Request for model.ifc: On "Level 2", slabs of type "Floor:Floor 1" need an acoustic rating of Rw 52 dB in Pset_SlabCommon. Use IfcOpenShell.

First a look at what the model holds.

```python
import ifcopenshell
import ifcopenshell.util.element

model = ifcopenshell.open("model.ifc")
print(model.schema)
storey = next(s for s in model.by_type("IfcBuildingStorey") if s.Name == "Level 2")
slabs = [e for e in ifcopenshell.util.element.get_decomposition(storey) if e.is_a("IfcSlab")]
seen = {}
for e in slabs:
    element_type = ifcopenshell.util.element.get_type(e)
    key = (element_type.Name if element_type != e and element_type else None, ifcopenshell.util.element.get_pset(e, "Pset_SlabCommon", "AcousticRating"))
    seen[key] = seen.get(key, 0) + 1
for (name, value), count in sorted(seen.items(), key=str):
    print(count, "x", name, "|", value)
```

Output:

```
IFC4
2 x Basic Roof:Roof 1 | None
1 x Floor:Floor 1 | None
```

```python
import ifcopenshell
import ifcopenshell.api.pset
import ifcopenshell.util.element

model = ifcopenshell.open("model.ifc")

storey = next(s for s in model.by_type("IfcBuildingStorey") if s.Name == "Level 2")
slabs = [e for e in ifcopenshell.util.element.get_decomposition(storey) if e.is_a("IfcSlab")]

count = 0
for e in slabs:
    element_type = ifcopenshell.util.element.get_type(e)
    if element_type in (None, e) or element_type.Name != "Floor:Floor 1":
        continue
    # add_pset returns the element's existing set when there is one.
    pset = ifcopenshell.api.pset.add_pset(model, product=e, name="Pset_SlabCommon")
    ifcopenshell.api.pset.edit_pset(model, pset=pset, properties={"AcousticRating": "Rw 52 dB"})
    count += 1

print(count, "slabs updated")

model.write("model_updated.ifc")
```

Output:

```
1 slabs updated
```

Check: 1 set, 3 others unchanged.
